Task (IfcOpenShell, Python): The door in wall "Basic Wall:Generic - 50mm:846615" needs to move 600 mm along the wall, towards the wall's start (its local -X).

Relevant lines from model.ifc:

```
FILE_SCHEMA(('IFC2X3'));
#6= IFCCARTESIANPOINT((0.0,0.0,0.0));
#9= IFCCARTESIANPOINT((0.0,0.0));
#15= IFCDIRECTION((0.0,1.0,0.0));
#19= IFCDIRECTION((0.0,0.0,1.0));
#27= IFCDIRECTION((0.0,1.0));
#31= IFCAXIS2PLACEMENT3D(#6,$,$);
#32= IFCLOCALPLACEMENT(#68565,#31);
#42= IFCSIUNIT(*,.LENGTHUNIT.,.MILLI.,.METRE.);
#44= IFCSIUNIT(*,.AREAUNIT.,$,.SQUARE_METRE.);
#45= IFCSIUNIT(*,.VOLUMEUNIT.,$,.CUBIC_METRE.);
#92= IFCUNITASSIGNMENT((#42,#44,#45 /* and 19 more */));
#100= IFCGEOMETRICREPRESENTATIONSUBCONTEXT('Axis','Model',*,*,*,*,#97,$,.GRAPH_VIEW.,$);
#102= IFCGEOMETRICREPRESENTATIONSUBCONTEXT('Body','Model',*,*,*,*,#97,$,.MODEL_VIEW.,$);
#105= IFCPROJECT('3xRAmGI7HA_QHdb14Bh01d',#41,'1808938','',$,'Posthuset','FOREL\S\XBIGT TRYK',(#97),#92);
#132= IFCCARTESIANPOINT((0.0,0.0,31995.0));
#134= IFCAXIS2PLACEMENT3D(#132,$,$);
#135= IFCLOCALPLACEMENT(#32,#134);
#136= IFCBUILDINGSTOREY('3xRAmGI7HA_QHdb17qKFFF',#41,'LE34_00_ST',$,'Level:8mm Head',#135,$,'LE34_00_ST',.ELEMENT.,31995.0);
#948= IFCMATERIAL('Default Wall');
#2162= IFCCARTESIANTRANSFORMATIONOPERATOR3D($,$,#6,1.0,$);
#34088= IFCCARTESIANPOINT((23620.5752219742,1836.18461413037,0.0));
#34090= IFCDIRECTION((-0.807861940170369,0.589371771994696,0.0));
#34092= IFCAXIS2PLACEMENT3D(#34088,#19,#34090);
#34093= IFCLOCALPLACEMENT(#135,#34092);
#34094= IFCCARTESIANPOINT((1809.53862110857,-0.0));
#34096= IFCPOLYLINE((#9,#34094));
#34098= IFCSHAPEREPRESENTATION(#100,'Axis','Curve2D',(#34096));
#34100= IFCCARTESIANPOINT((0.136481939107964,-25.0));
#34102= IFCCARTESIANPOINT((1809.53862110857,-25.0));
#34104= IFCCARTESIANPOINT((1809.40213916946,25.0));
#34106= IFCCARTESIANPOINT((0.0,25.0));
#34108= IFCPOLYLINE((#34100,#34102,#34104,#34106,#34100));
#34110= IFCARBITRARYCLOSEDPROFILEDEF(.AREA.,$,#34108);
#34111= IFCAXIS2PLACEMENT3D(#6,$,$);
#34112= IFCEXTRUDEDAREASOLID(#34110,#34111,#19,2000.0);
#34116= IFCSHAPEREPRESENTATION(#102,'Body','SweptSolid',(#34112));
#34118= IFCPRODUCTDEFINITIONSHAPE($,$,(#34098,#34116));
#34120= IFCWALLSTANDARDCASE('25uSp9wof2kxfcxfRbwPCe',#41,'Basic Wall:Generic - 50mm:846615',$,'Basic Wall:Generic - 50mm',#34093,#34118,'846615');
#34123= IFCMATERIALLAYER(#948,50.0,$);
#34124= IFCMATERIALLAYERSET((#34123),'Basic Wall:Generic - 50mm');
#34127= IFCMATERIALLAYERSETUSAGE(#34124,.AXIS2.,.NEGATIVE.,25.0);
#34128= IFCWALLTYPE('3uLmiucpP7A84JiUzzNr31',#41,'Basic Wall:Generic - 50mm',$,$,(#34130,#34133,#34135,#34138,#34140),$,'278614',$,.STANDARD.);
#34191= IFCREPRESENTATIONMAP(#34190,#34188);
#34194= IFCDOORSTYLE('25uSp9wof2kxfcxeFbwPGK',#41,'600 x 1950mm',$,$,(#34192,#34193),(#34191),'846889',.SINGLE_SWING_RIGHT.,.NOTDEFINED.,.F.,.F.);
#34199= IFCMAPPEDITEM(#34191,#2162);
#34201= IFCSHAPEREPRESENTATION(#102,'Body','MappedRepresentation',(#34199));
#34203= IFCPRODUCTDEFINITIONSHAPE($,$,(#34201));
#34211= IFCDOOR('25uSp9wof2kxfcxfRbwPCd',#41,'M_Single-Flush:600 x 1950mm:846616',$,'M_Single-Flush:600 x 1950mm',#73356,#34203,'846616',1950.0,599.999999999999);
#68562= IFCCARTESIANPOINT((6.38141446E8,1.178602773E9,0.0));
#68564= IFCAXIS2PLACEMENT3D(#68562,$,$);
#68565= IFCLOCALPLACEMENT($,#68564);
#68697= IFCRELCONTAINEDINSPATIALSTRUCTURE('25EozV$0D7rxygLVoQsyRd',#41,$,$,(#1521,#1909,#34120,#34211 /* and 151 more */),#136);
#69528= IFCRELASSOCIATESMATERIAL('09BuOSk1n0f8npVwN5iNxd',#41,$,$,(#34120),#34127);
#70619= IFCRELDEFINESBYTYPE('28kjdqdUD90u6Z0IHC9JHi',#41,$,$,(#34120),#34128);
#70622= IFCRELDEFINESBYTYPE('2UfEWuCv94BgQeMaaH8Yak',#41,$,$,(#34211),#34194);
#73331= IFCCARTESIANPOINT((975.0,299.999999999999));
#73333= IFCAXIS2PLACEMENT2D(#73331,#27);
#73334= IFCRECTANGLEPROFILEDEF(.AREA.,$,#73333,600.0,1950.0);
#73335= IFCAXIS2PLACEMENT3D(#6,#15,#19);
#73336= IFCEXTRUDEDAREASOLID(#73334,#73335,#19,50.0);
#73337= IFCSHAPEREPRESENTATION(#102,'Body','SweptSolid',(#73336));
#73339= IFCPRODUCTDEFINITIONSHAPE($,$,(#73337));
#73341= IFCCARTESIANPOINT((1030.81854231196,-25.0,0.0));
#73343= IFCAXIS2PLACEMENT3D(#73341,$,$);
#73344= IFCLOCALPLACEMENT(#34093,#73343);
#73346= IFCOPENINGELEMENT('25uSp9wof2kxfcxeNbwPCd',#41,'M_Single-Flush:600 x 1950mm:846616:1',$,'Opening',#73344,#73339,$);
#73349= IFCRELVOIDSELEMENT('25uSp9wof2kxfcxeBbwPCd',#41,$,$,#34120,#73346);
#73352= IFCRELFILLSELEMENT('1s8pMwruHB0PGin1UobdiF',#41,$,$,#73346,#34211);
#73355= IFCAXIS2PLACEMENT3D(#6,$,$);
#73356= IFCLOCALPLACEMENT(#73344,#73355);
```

```python
import ifcopenshell
import ifcopenshell.api.geometry
import ifcopenshell.util.placement

model = ifcopenshell.open("model.ifc")

door = model.by_guid("25uSp9wof2kxfcxfRbwPCd")
opening = door.FillsVoids[0].RelatingOpeningElement
wall = opening.VoidsElements[0].RelatingBuildingElement

wall_matrix = ifcopenshell.util.placement.get_local_placement(wall.ObjectPlacement)
shift = wall_matrix[:3, 0] * -600.0
before = ifcopenshell.util.placement.get_local_placement(door.ObjectPlacement)[:3, 3].copy()

# The door is placed relative to its opening, so it follows when the opening moves.
matrix = ifcopenshell.util.placement.get_local_placement(opening.ObjectPlacement)
matrix[:3, 3] += shift
ifcopenshell.api.geometry.edit_object_placement(
    model, product=opening, matrix=matrix, is_si=False, should_transform_children=True
)

after = ifcopenshell.util.placement.get_local_placement(door.ObjectPlacement)[:3, 3]
print("door moved by", (after - before).round(3) + 0.0)

model.write("model_edited.ifc")
```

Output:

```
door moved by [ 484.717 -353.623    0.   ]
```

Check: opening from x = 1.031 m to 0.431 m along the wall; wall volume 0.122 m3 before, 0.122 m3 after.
